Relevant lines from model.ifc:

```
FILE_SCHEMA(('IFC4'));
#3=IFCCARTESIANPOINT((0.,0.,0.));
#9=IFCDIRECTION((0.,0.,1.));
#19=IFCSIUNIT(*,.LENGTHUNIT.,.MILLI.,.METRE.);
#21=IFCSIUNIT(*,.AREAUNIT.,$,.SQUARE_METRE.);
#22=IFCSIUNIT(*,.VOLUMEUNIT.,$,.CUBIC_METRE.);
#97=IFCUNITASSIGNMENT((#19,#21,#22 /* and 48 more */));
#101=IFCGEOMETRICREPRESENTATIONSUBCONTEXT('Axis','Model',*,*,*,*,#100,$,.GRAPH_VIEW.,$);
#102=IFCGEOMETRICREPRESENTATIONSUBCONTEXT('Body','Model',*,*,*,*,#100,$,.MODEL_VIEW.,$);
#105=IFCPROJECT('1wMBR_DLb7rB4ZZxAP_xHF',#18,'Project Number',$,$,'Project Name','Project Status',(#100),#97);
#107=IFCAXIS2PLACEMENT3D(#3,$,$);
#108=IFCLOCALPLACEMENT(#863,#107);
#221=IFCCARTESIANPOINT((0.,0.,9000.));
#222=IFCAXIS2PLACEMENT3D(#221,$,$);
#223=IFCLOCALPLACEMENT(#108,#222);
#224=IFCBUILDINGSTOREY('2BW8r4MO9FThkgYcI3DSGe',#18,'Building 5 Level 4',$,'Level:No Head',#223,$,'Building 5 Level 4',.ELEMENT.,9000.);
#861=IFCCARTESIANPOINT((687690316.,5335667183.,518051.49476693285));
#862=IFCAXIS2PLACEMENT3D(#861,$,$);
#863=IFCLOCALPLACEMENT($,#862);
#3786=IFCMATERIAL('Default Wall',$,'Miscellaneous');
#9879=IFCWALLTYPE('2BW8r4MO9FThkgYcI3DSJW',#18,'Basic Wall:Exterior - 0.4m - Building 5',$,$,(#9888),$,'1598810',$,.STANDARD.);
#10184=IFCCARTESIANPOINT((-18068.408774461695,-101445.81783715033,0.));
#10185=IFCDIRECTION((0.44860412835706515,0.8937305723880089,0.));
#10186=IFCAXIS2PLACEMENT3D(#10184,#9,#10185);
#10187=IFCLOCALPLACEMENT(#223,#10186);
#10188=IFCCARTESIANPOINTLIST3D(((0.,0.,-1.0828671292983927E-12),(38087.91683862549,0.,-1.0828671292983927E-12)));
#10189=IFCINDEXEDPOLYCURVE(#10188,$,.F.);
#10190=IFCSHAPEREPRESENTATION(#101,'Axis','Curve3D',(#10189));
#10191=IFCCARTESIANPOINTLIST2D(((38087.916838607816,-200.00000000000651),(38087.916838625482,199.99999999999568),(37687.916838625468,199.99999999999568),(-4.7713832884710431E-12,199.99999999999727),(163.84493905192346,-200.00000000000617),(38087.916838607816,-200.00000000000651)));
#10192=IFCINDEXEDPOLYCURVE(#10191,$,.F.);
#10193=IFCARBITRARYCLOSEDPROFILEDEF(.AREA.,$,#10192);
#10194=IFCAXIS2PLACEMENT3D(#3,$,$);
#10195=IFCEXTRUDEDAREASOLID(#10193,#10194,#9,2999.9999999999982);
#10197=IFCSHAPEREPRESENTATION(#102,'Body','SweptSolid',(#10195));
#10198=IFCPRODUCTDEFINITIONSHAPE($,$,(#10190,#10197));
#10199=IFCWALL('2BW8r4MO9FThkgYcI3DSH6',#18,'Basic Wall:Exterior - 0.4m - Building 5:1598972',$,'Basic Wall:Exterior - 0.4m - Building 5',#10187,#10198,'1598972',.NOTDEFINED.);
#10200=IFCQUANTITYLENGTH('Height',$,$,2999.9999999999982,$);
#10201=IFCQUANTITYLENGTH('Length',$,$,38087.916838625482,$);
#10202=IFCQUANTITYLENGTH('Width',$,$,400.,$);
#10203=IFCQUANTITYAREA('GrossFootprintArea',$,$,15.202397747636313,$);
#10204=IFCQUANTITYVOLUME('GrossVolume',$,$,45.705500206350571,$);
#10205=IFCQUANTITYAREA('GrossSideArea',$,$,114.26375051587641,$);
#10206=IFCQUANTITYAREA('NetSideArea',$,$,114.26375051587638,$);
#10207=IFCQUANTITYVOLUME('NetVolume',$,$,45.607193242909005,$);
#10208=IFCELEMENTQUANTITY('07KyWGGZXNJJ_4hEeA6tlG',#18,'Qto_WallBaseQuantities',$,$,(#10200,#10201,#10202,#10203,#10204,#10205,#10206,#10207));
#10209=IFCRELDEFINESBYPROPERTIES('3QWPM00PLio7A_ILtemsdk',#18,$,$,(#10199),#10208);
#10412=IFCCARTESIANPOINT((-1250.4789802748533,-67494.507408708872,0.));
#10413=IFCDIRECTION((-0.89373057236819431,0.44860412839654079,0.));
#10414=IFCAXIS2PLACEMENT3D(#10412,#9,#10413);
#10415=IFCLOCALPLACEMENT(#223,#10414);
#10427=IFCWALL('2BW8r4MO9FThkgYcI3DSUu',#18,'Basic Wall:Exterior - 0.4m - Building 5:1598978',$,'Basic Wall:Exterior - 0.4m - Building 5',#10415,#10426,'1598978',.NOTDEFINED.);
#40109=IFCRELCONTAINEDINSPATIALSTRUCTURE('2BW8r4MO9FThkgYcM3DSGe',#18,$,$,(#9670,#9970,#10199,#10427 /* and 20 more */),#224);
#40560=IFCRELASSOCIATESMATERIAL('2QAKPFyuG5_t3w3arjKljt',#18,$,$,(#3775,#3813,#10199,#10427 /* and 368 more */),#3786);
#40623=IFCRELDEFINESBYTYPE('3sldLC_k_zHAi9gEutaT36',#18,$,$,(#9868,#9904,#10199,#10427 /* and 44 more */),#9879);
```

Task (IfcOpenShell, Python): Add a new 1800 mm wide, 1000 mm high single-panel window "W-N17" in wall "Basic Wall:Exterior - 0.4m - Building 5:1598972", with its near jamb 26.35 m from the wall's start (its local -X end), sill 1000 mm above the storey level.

```python
import numpy as np
import ifcopenshell
import ifcopenshell.api.feature
import ifcopenshell.api.geometry
import ifcopenshell.api.pset
import ifcopenshell.api.root
import ifcopenshell.api.spatial
import ifcopenshell.geom
import ifcopenshell.util.element
import ifcopenshell.util.placement
import ifcopenshell.util.representation
import ifcopenshell.util.shape
import ifcopenshell.util.unit

model = ifcopenshell.open("model.ifc")
unit_scale = ifcopenshell.util.unit.calculate_unit_scale(model)
area_scale = ifcopenshell.util.unit.calculate_unit_scale(model, "AREAUNIT")
volume_scale = ifcopenshell.util.unit.calculate_unit_scale(model, "VOLUMEUNIT")
settings = ifcopenshell.geom.settings()


def volume(element):
    """Net volume in cubic metres, openings subtracted."""
    shape = ifcopenshell.geom.create_shape(settings, element)
    return ifcopenshell.util.shape.get_volume(shape.geometry)


wall = model.by_id(10199)
storey = ifcopenshell.util.element.get_container(wall, ifc_class="IfcBuildingStorey")
context = ifcopenshell.util.representation.get_context(model, "Model", "Body", "MODEL_VIEW")
before = volume(wall)

width, height, from_end, sill = 1.8, 1, 26.35, 1  # metres

# The wall runs along its own X axis, and the end named is its -X end.
wall_shape = ifcopenshell.geom.create_shape(settings, wall)
x, y, z = ifcopenshell.util.shape.get_vertices(wall_shape.geometry).T
start = x.min() + from_end
face, thickness = float(y.min()), float(y.max() - y.min())
wall_matrix = ifcopenshell.util.placement.get_local_placement(wall.ObjectPlacement)
level = ifcopenshell.util.placement.get_local_placement(storey.ObjectPlacement)[2, 3]


def in_wall(x, y):
    """Placement at x, y metres in the wall's axes, at sill height."""
    matrix = wall_matrix.copy()
    matrix[:, 3] = wall_matrix @ np.array([x / unit_scale, y / unit_scale, 0.0, 1.0])
    matrix[2, 3] = level + sill / unit_scale
    return matrix


# Opening: a box that overshoots both wall faces by 50 mm.
opening = ifcopenshell.api.root.create_entity(model, ifc_class="IfcOpeningElement", predefined_type="OPENING")
box = ifcopenshell.api.geometry.add_wall_representation(
    model, context=context, length=width, height=height, thickness=thickness + 0.1
)
ifcopenshell.api.geometry.assign_representation(model, product=opening, representation=box)
ifcopenshell.api.geometry.edit_object_placement(model, product=opening, matrix=in_wall(start, face - 0.05), is_si=False)
ifcopenshell.api.feature.add_feature(model, feature=opening, element=wall)

window = ifcopenshell.api.root.create_entity(model, ifc_class="IfcWindow", name="W-N17", predefined_type="WINDOW")
window.OverallWidth, window.OverallHeight = width / unit_scale, height / unit_scale
window.PartitioningType = "SINGLE_PANEL"
body = ifcopenshell.api.geometry.add_window_representation(
    model,
    context=context,
    overall_width=window.OverallWidth,
    overall_height=window.OverallHeight,
    partition_type="SINGLE_PANEL",
)
ifcopenshell.api.geometry.assign_representation(model, product=window, representation=body)
ifcopenshell.api.spatial.assign_container(model, products=[window], relating_structure=storey)
ifcopenshell.api.feature.add_filling(model, opening=opening, element=window)

# Centre the window in the wall's thickness.
ifcopenshell.api.geometry.edit_object_placement(model, product=window, matrix=in_wall(start, face), is_si=False)
window_shape = ifcopenshell.geom.create_shape(settings, window)
depth = ifcopenshell.util.shape.get_vertices(window_shape.geometry)[:, 1]
offset = face + thickness / 2 - (depth.min() + depth.max()) / 2
ifcopenshell.api.geometry.edit_object_placement(model, product=window, matrix=in_wall(start, offset), is_si=False)

after = volume(wall)

# Update the wall's stored quantities.
qto = model.by_id(ifcopenshell.util.element.get_pset(wall, "Qto_WallBaseQuantities", should_inherit=False)["id"])
ifcopenshell.api.pset.edit_qto(model, qto=qto, properties={
    "NetSideArea": after / thickness / area_scale,
    "NetVolume": after / volume_scale,
})

print(f"wall volume {before:.3f} -> {after:.3f} m3")

model.write("model_updated.ifc")
```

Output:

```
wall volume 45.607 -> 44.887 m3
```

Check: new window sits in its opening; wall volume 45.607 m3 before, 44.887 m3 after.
